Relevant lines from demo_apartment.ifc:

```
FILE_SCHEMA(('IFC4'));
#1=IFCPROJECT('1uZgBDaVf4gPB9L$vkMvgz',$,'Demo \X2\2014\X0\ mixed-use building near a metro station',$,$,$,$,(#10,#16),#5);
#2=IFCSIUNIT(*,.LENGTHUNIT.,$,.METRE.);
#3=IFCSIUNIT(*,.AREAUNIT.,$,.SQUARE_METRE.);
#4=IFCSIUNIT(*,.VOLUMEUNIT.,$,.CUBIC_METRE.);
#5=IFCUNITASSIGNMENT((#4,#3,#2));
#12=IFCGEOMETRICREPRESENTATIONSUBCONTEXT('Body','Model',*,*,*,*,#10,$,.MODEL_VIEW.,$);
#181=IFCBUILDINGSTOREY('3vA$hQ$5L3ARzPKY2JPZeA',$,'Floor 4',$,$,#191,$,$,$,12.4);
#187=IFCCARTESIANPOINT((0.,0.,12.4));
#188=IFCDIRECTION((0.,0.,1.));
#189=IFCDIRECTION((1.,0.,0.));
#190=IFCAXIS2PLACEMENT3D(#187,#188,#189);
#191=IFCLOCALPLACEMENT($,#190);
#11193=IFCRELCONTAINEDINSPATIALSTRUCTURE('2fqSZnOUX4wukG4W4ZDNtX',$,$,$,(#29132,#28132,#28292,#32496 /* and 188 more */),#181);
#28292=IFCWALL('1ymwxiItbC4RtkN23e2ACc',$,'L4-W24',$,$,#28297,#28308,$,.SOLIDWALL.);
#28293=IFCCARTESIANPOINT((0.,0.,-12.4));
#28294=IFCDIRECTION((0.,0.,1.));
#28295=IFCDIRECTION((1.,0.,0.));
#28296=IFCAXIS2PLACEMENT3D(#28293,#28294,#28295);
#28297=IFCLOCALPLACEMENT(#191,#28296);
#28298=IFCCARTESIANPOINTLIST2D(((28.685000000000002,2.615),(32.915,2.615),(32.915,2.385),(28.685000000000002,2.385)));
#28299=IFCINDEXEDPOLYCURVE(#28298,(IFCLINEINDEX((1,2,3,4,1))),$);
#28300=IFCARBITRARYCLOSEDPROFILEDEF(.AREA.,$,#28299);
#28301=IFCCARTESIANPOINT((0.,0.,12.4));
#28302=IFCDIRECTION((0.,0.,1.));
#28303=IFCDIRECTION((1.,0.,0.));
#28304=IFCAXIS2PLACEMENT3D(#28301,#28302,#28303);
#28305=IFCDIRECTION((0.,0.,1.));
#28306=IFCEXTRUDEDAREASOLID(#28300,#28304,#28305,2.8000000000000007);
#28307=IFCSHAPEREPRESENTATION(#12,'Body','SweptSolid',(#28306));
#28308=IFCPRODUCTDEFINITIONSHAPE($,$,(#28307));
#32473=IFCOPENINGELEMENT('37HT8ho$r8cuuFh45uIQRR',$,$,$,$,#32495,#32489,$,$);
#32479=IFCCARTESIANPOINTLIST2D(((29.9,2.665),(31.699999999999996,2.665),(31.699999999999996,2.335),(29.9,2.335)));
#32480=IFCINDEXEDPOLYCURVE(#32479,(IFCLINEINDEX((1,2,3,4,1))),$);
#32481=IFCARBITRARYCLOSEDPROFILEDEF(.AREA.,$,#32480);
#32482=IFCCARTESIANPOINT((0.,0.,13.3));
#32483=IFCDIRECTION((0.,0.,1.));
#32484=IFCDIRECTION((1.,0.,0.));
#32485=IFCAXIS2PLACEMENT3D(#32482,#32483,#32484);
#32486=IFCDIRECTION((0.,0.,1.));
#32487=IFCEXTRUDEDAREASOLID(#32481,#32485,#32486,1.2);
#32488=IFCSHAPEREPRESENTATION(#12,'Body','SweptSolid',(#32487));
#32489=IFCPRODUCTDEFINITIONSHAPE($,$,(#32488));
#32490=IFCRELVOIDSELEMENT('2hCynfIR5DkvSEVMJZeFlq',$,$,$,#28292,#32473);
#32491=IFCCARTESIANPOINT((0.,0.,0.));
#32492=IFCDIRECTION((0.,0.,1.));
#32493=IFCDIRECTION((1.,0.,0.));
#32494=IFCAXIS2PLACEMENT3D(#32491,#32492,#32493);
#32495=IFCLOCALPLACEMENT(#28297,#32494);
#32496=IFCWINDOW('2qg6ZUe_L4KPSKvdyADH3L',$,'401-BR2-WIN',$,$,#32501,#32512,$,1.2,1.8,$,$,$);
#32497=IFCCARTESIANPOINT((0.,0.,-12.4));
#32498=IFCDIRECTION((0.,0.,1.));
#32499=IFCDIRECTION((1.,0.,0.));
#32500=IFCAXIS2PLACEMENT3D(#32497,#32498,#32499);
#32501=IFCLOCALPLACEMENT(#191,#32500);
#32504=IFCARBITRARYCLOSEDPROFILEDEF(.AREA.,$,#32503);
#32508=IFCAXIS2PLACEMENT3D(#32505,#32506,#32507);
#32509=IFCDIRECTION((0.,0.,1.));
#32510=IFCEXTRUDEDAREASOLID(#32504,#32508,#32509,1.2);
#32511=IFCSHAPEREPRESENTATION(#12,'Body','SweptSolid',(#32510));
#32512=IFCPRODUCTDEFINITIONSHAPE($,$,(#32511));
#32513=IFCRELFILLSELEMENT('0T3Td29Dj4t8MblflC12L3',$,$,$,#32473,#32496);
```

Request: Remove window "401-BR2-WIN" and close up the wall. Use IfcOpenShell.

```python
import ifcopenshell
import ifcopenshell.api.feature
import ifcopenshell.api.root
import ifcopenshell.geom
import ifcopenshell.util.shape

model = ifcopenshell.open("demo_apartment.ifc")
settings = ifcopenshell.geom.settings()


def volume(element):
    """Net volume in cubic metres, openings subtracted."""
    shape = ifcopenshell.geom.create_shape(settings, element)
    return ifcopenshell.util.shape.get_volume(shape.geometry)


window = model.by_guid("2qg6ZUe_L4KPSKvdyADH3L")
opening = window.FillsVoids[0].RelatingOpeningElement
wall = opening.VoidsElements[0].RelatingBuildingElement
before = volume(wall)

ifcopenshell.api.root.remove_product(model, product=window)
ifcopenshell.api.feature.remove_feature(model, feature=opening)

after = volume(wall)

print(f"wall volume {before:.3f} -> {after:.3f} m3")

model.write("demo_apartment-out.ifc")
```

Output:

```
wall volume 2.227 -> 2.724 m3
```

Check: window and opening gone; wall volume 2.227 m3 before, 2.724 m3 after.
